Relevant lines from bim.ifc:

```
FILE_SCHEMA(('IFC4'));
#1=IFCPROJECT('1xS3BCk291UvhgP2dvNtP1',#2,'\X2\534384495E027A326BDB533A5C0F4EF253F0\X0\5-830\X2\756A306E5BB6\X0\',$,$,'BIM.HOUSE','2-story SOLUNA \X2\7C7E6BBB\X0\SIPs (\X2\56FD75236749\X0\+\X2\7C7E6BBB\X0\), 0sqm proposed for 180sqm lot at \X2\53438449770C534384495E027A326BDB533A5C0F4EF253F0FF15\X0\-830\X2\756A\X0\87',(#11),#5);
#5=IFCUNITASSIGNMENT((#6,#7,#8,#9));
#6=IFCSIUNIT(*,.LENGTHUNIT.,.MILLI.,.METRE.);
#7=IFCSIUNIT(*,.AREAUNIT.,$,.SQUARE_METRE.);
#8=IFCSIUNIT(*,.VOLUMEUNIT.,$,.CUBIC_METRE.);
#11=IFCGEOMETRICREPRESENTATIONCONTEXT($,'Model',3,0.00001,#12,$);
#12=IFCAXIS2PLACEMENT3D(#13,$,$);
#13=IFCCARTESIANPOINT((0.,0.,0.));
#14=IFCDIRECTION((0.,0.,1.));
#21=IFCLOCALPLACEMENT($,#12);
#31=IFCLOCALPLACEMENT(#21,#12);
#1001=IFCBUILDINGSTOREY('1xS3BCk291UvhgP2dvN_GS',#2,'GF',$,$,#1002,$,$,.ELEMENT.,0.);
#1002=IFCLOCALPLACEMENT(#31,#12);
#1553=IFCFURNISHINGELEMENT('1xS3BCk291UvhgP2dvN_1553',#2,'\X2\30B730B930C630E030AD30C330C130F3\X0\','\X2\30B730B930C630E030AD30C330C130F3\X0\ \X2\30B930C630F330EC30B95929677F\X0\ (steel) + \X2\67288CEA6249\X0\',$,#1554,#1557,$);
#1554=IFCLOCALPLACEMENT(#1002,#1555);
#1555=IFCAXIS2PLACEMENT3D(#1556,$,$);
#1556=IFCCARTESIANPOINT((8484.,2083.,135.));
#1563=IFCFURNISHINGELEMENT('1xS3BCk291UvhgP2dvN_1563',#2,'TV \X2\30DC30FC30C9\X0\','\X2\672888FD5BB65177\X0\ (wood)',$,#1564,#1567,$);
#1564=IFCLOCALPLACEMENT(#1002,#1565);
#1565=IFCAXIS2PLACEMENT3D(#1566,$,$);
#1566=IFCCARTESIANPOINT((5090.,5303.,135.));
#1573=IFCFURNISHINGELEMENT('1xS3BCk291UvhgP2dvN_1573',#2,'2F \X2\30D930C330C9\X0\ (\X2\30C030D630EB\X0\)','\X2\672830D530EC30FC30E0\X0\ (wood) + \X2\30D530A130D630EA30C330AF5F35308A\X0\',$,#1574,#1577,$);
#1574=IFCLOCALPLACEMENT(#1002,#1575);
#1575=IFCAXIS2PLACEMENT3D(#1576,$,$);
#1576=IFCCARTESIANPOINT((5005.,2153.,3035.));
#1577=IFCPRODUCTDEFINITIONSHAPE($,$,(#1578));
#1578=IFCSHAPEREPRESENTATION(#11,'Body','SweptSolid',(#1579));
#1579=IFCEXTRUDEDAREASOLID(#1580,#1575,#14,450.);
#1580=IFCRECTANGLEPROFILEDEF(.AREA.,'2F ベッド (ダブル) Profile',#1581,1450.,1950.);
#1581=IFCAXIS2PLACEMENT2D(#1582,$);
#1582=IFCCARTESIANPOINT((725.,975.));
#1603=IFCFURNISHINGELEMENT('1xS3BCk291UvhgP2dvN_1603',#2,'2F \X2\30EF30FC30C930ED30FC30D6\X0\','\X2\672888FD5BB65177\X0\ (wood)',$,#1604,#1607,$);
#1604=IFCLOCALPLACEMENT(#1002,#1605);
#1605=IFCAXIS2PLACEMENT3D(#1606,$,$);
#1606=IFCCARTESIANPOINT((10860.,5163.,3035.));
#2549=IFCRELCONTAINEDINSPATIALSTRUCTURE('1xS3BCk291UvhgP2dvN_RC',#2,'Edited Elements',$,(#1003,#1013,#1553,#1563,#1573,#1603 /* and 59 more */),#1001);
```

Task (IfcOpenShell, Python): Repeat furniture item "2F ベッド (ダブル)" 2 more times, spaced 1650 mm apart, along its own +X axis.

```python
import ifcopenshell
import ifcopenshell.api.geometry
import ifcopenshell.api.root
import ifcopenshell.util.element
import ifcopenshell.util.placement
import ifcopenshell.util.unit

model = ifcopenshell.open("bim.ifc")
unit_scale = ifcopenshell.util.unit.calculate_unit_scale(model)


def reuse_history(source, copy):
    """copy_class also copies each property set's owner history, people and application; keep the originals."""
    for rel in copy.IsDefinedBy:
        if rel.is_a("IfcRelDefinesByProperties") and (history := rel.RelatingPropertyDefinition.OwnerHistory):
            rel.RelatingPropertyDefinition.OwnerHistory = source.OwnerHistory
            ifcopenshell.util.element.remove_deep2(model, history)


source = model.by_guid("1xS3BCk291UvhgP2dvN_1573")
base = ifcopenshell.util.placement.get_local_placement(source.ObjectPlacement)
step = base[:3, 0] * 1.65 / unit_scale

for i in range(1, 3):
    copy = ifcopenshell.api.root.copy_class(model, product=source)
    copy.Representation = ifcopenshell.util.element.copy_deep(
        model, source.Representation, exclude=["IfcGeometricRepresentationContext", "IfcRepresentationMap"]
    )
    reuse_history(source, copy)
    matrix = base.copy()
    matrix[:3, 3] += i * step
    print("added at", matrix[:3, 3].round(3) + 0.0)
    ifcopenshell.api.geometry.edit_object_placement(model, product=copy, matrix=matrix, is_si=False)

model.write("bim-out.ifc")
```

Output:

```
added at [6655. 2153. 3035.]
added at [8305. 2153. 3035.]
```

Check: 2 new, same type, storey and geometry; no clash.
